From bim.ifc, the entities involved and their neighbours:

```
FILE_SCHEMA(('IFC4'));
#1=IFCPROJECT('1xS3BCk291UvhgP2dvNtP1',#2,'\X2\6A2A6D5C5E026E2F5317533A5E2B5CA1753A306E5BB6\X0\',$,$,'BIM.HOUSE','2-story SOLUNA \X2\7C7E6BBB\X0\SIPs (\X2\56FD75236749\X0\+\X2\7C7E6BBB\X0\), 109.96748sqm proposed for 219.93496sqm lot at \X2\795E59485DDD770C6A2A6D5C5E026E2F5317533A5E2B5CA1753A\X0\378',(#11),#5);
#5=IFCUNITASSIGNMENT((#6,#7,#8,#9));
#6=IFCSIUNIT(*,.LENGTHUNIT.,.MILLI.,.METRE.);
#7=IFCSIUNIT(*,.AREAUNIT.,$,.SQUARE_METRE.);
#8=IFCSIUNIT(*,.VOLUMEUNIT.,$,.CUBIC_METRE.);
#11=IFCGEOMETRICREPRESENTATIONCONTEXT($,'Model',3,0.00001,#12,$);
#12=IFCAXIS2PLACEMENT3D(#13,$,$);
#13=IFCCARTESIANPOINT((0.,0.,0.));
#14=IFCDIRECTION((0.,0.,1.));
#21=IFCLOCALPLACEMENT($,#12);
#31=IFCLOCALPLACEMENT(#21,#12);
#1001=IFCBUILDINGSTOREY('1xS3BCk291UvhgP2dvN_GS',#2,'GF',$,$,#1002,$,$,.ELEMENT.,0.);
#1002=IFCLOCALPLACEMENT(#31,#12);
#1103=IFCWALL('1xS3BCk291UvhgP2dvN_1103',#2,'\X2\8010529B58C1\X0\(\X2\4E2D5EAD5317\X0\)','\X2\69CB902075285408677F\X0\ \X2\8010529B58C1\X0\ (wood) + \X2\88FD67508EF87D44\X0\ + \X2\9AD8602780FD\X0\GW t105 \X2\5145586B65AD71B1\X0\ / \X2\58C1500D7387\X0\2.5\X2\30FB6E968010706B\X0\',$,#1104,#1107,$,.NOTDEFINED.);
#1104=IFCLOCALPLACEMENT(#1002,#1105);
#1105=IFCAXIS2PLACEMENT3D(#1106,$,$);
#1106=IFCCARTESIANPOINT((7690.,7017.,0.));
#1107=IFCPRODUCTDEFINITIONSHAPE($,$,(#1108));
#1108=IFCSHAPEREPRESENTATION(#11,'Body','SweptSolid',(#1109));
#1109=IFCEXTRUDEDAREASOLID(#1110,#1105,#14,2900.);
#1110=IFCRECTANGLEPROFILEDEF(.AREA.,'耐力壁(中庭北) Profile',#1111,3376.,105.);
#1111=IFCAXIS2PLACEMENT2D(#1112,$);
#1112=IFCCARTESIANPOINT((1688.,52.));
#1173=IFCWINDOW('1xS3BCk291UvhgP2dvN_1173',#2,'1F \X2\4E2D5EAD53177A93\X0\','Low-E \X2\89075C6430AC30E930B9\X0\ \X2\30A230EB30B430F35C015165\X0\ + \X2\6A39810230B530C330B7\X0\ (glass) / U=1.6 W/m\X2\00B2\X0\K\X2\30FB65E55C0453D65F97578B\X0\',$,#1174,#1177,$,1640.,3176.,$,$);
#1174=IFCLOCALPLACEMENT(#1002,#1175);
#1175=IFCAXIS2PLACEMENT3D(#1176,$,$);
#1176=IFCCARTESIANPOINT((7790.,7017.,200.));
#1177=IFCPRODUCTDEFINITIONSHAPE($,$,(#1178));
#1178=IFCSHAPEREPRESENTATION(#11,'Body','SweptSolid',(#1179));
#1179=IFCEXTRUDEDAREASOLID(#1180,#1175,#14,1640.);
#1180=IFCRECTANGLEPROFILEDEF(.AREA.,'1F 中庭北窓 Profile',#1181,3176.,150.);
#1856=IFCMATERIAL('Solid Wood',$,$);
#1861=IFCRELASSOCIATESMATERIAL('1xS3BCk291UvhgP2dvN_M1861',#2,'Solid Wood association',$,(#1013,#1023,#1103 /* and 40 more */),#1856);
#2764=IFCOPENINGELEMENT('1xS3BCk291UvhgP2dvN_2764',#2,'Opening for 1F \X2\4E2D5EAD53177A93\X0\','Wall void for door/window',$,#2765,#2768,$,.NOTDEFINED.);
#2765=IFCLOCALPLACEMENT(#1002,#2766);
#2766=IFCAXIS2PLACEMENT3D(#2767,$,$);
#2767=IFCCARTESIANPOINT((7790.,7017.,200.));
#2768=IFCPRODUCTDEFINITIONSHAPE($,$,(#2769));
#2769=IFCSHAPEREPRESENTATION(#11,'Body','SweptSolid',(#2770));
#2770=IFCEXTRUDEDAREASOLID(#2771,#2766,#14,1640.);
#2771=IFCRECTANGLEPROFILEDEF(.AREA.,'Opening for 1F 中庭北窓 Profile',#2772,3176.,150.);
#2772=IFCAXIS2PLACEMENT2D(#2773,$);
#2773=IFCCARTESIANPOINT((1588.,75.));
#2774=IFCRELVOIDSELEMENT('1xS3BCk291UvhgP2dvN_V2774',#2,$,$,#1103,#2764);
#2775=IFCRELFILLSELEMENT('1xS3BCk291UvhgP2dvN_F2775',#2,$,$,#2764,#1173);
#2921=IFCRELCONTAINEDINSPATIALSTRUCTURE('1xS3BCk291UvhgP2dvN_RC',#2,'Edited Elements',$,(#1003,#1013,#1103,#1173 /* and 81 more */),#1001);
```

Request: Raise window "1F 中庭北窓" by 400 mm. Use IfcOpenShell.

```python
import numpy as np
import ifcopenshell
import ifcopenshell.api.geometry
import ifcopenshell.util.placement
import ifcopenshell.util.unit

model = ifcopenshell.open("bim.ifc")
unit_scale = ifcopenshell.util.unit.calculate_unit_scale(model)

window = model.by_guid("1xS3BCk291UvhgP2dvN_1173")
opening = window.FillsVoids[0].RelatingOpeningElement
dz = 400.0

shift = np.array([0.0, 0.0, dz])
# The window is not placed relative to its opening, so move both.
for product in (opening, window):
    matrix = ifcopenshell.util.placement.get_local_placement(product.ObjectPlacement)
    matrix[:3, 3] += shift
    ifcopenshell.api.geometry.edit_object_placement(model, product=product, matrix=matrix, is_si=False)

print(f"moved by {dz * unit_scale:+.3f} m")

model.write("bim_updated.ifc")
```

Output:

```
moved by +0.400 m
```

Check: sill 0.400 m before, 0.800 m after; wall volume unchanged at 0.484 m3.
